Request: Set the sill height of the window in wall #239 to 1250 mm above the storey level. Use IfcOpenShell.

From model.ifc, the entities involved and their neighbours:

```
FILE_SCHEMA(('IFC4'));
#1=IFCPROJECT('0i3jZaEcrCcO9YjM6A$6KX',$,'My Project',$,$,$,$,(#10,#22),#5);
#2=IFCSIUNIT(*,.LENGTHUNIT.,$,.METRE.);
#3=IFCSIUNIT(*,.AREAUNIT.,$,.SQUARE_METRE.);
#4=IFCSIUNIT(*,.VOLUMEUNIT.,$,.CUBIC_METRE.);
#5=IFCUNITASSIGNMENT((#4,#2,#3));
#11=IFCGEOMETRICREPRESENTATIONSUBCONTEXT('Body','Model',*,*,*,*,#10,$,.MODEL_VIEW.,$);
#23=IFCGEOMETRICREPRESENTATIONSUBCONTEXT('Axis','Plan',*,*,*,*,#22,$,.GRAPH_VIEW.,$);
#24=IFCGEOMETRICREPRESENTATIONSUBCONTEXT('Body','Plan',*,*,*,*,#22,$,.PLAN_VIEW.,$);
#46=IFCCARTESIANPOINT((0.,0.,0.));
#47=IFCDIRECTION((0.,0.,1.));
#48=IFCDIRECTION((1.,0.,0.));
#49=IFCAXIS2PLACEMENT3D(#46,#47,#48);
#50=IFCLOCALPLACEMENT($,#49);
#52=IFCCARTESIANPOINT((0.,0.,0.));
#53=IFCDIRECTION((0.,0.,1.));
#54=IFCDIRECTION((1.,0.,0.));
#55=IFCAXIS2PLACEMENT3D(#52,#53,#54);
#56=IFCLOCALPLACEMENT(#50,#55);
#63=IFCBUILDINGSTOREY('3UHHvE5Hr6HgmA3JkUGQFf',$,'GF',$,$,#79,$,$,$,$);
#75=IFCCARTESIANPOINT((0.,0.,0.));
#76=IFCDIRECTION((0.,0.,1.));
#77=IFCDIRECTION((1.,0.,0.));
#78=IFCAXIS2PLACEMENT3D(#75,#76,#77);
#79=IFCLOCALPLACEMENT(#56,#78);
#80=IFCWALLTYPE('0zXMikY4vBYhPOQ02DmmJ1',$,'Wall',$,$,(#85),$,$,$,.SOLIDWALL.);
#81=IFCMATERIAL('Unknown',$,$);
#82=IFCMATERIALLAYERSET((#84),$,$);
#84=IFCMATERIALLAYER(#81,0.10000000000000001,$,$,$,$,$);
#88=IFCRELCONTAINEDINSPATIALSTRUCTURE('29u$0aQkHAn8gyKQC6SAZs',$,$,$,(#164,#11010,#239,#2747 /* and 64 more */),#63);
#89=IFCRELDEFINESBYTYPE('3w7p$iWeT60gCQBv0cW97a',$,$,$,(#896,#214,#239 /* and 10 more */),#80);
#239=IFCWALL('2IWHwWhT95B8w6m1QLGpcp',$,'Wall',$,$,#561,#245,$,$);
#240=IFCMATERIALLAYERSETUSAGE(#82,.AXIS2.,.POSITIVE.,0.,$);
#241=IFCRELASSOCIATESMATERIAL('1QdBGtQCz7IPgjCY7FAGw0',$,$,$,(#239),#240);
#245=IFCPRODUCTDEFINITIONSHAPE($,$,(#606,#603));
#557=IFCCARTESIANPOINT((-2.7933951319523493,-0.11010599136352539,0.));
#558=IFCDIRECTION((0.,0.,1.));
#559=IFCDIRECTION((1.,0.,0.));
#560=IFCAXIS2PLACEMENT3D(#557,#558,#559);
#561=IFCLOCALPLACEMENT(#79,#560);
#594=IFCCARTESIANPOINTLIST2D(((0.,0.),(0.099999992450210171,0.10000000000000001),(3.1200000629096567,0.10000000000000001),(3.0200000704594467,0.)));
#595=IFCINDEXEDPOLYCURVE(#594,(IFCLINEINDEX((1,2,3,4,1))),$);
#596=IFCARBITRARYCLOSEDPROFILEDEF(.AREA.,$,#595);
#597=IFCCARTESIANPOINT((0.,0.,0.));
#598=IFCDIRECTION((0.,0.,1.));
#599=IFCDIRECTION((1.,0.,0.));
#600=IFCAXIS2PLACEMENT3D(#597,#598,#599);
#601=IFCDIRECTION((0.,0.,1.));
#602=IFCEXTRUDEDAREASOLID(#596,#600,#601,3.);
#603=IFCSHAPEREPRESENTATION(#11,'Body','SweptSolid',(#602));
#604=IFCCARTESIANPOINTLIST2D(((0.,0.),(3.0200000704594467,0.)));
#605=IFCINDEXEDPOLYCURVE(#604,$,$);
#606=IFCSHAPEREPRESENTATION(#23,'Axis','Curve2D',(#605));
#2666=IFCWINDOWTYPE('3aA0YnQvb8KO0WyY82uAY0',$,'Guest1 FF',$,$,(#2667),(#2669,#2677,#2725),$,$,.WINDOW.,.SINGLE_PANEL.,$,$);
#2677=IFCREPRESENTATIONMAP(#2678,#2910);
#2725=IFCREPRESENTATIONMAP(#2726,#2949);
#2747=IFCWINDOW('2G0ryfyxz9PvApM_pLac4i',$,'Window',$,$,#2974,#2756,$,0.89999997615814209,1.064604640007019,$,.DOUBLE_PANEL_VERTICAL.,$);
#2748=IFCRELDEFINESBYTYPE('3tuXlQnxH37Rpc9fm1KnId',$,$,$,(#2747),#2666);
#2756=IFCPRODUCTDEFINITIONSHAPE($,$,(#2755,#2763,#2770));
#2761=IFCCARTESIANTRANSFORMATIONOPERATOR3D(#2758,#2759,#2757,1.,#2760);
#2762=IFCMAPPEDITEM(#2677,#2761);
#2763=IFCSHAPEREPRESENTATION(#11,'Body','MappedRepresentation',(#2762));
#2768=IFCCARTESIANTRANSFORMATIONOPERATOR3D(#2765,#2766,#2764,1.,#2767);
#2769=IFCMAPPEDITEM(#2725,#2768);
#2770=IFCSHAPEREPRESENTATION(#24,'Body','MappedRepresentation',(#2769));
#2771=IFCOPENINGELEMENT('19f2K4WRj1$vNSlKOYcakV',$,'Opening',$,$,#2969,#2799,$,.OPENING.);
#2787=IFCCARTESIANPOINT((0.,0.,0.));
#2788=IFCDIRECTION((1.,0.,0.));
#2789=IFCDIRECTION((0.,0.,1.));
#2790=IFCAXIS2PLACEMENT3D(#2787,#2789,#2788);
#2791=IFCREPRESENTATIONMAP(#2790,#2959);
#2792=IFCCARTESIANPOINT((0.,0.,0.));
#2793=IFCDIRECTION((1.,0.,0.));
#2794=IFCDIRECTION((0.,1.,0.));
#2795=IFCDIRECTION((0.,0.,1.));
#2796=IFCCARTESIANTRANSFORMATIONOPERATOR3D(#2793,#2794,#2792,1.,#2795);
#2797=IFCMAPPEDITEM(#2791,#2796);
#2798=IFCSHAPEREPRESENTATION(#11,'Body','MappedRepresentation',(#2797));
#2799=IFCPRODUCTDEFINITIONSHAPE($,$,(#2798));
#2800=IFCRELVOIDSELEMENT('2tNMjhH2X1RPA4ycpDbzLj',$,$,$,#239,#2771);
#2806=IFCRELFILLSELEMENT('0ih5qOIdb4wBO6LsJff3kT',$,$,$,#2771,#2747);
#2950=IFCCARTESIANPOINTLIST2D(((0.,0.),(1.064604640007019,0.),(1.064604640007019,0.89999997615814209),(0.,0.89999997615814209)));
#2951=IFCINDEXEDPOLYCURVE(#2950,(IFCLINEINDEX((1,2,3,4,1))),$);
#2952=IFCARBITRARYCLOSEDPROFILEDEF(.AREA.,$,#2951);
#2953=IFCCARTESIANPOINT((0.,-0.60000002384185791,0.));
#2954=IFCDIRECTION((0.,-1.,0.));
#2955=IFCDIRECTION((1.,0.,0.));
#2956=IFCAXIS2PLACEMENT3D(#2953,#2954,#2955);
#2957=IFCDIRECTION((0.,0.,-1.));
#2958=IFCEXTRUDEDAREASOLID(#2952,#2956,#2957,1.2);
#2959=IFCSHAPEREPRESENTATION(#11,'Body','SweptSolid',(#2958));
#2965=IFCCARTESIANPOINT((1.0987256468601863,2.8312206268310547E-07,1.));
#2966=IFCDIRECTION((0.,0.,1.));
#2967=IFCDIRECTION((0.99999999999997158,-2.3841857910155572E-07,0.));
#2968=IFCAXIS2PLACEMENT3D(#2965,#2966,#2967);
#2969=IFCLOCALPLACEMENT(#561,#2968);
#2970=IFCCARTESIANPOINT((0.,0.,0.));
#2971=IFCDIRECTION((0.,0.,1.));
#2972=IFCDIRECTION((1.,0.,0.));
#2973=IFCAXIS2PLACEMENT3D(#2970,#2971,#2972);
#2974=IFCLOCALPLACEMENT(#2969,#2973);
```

```python
import numpy as np
import ifcopenshell
import ifcopenshell.api.geometry
import ifcopenshell.geom
import ifcopenshell.util.element
import ifcopenshell.util.placement
import ifcopenshell.util.shape
import ifcopenshell.util.unit

model = ifcopenshell.open("model.ifc")
unit_scale = ifcopenshell.util.unit.calculate_unit_scale(model)

window = model.by_id(2747)
opening = window.FillsVoids[0].RelatingOpeningElement
storey = ifcopenshell.util.element.get_container(window, ifc_class="IfcBuildingStorey")
level = ifcopenshell.util.placement.get_local_placement(storey.ObjectPlacement)[2, 3]

# The opening's origin need not be at the sill, so measure its lowest point.
shape = ifcopenshell.geom.create_shape(ifcopenshell.geom.settings(), opening)
bottom = ifcopenshell.util.shape.get_shape_bottom_elevation(shape, shape.geometry) / unit_scale
dz = level + 1.25 / unit_scale - bottom

shift = np.array([0.0, 0.0, dz])
# The window is placed relative to its opening, so it follows when the opening moves.
matrix = ifcopenshell.util.placement.get_local_placement(opening.ObjectPlacement)
matrix[:3, 3] += shift
ifcopenshell.api.geometry.edit_object_placement(
    model, product=opening, matrix=matrix, is_si=False, should_transform_children=True
)

print(f"moved by {dz * unit_scale:+.3f} m")

model.write("model_updated.ifc")
```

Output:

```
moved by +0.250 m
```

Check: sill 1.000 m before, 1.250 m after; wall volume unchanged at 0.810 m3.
